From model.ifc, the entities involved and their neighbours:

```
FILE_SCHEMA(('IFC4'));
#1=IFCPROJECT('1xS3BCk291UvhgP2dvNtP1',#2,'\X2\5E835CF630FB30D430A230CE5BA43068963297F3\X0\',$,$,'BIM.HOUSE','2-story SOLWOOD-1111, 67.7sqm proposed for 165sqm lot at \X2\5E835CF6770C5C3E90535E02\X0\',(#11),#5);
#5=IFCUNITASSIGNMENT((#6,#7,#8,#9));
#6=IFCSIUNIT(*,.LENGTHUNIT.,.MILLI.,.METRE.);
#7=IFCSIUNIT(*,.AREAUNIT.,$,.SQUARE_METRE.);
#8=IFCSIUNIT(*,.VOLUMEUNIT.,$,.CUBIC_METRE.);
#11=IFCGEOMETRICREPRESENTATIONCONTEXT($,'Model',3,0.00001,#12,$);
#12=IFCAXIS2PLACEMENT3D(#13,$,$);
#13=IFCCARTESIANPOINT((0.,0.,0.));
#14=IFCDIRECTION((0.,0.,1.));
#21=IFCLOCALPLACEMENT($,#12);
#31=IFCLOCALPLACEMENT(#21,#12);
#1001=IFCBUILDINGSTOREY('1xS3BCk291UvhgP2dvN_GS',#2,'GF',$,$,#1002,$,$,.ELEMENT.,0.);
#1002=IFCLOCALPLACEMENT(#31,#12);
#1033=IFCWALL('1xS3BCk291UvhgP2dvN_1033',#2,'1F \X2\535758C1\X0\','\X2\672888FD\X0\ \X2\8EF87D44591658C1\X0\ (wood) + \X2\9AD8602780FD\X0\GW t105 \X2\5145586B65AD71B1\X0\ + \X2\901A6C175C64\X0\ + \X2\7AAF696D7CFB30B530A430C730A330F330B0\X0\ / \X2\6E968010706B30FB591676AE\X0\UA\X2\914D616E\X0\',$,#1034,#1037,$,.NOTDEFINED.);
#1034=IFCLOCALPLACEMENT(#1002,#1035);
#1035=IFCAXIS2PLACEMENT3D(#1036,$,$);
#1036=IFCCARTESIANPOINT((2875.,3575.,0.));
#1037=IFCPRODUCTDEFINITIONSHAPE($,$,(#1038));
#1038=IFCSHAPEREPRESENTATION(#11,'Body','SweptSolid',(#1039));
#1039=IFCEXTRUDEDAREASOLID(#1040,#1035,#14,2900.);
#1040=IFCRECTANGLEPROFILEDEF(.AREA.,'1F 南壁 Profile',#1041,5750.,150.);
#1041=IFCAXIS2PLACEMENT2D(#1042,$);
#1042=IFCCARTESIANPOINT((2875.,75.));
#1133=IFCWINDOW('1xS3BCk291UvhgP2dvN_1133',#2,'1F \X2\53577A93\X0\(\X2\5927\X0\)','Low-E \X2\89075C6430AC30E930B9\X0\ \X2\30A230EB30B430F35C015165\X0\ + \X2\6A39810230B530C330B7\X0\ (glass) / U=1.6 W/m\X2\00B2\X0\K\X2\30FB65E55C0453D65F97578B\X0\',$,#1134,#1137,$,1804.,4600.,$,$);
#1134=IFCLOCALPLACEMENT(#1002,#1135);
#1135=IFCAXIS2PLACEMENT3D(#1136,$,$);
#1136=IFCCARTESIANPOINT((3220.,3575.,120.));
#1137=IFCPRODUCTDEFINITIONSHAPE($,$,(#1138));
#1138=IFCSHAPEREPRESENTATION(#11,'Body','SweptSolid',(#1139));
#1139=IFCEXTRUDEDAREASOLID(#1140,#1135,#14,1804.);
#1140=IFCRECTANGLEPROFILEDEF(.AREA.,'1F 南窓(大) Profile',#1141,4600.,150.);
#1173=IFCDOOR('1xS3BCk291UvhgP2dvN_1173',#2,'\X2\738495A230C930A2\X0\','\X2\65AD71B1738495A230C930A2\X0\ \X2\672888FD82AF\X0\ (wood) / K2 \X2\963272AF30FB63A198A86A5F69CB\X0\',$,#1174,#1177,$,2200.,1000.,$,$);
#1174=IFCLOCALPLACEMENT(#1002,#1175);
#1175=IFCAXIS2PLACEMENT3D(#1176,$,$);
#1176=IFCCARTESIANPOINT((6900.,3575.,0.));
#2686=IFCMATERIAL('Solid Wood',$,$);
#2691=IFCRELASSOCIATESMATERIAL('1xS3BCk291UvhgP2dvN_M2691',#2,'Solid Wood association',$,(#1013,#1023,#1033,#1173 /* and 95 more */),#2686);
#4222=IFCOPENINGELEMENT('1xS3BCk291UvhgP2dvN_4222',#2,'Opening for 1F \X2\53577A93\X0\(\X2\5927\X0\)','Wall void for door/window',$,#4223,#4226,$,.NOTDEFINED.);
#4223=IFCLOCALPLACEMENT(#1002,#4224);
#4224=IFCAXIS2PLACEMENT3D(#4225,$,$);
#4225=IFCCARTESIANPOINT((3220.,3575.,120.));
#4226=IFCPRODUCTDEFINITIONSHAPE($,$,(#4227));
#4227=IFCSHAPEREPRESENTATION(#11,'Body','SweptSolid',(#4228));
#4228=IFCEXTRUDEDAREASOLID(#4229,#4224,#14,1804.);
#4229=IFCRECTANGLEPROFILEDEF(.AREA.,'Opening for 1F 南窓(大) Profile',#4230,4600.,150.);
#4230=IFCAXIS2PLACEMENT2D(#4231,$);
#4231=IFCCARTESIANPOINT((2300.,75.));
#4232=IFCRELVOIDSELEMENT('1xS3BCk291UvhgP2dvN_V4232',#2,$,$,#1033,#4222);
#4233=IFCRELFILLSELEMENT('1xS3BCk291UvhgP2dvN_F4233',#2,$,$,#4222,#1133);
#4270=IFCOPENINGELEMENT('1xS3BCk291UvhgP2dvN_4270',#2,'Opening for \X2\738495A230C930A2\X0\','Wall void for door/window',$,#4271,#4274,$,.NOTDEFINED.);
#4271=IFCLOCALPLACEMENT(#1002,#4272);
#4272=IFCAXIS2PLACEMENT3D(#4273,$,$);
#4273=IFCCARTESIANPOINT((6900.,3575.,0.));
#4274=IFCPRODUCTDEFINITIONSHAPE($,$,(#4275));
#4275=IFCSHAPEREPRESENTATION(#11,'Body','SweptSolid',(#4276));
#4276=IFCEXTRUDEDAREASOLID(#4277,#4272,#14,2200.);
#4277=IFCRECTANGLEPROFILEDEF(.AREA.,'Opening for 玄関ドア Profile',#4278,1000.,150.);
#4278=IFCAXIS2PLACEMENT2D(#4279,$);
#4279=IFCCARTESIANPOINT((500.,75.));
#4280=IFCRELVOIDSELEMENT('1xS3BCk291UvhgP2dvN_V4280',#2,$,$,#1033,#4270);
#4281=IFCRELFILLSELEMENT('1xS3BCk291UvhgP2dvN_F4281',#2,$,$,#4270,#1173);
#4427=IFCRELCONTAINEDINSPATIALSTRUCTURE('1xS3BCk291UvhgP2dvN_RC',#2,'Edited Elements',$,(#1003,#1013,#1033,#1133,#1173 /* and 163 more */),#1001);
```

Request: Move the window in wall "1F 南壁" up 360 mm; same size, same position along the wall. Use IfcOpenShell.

```python
import numpy as np
import ifcopenshell
import ifcopenshell.api.geometry
import ifcopenshell.util.placement
import ifcopenshell.util.unit

model = ifcopenshell.open("model.ifc")
unit_scale = ifcopenshell.util.unit.calculate_unit_scale(model)

window = model.by_guid("1xS3BCk291UvhgP2dvN_1133")
opening = window.FillsVoids[0].RelatingOpeningElement
dz = 360.0

shift = np.array([0.0, 0.0, dz])
# The window is not placed relative to its opening, so move both.
for product in (opening, window):
    matrix = ifcopenshell.util.placement.get_local_placement(product.ObjectPlacement)
    matrix[:3, 3] += shift
    ifcopenshell.api.geometry.edit_object_placement(model, product=product, matrix=matrix, is_si=False)

print(f"moved by {dz * unit_scale:+.3f} m")

model.write("model_v2.ifc")
```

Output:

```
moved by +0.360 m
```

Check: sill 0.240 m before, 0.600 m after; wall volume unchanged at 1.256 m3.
